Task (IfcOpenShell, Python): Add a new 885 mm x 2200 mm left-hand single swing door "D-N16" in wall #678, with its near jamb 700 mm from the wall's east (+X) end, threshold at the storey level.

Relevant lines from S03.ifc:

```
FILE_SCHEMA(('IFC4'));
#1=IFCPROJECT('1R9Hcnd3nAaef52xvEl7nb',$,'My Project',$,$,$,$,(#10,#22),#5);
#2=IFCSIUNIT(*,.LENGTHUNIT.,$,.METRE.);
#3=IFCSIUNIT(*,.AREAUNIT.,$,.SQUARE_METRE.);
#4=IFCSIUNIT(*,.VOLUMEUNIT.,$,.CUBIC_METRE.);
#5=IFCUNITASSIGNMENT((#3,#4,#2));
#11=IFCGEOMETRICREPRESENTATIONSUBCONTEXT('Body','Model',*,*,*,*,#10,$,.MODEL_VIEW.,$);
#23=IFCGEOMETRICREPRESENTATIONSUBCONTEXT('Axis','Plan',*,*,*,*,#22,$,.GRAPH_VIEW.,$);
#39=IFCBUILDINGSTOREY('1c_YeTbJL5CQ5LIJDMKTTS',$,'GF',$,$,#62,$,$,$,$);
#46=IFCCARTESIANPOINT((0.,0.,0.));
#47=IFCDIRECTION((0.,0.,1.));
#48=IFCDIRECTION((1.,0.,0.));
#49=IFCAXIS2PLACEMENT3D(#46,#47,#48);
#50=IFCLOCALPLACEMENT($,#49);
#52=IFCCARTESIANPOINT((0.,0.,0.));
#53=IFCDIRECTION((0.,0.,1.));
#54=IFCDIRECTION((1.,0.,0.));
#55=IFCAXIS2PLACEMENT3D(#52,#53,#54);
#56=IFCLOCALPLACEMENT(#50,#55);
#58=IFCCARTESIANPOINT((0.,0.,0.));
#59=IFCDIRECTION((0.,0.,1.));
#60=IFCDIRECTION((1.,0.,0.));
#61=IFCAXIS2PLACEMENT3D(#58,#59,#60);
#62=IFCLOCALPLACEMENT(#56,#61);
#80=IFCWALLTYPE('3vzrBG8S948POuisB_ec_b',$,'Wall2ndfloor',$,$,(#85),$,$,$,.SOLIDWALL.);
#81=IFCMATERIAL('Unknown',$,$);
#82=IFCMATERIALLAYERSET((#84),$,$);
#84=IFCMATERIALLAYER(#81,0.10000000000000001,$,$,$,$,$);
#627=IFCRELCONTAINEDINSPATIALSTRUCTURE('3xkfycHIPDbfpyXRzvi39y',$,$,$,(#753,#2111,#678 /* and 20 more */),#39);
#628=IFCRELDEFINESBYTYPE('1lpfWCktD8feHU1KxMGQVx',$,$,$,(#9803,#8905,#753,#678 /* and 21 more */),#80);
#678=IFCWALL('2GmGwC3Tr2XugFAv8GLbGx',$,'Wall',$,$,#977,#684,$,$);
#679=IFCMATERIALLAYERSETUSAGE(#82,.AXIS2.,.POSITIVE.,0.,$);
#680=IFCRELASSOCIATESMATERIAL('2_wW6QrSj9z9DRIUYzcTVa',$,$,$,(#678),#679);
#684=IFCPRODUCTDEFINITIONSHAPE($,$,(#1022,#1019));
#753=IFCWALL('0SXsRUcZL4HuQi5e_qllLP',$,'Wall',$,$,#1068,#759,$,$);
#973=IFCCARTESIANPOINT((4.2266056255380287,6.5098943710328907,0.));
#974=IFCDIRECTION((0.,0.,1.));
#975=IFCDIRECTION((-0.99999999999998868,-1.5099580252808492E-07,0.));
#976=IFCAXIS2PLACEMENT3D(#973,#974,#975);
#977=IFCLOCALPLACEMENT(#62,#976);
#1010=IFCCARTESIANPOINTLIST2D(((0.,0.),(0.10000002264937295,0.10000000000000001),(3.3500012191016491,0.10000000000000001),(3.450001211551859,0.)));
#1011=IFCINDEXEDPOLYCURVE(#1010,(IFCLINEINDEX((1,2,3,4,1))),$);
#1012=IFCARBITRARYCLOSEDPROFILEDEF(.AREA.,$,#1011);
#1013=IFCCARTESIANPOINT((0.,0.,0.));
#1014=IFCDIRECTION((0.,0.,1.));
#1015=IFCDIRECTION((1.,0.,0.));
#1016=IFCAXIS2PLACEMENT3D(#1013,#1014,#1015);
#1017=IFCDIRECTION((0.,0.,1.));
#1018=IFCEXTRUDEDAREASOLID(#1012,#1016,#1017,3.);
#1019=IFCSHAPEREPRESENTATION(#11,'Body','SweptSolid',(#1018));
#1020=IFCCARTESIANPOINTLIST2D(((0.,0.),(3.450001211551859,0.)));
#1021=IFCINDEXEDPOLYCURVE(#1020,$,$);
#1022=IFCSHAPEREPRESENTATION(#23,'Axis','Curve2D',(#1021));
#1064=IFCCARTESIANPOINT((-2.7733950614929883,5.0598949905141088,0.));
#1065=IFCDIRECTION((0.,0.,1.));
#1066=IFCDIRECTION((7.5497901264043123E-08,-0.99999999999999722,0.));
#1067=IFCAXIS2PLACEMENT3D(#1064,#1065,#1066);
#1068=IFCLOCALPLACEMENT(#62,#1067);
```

```python
import numpy as np
import ifcopenshell
import ifcopenshell.api.feature
import ifcopenshell.api.geometry
import ifcopenshell.api.root
import ifcopenshell.api.spatial
import ifcopenshell.geom
import ifcopenshell.util.element
import ifcopenshell.util.placement
import ifcopenshell.util.representation
import ifcopenshell.util.shape
import ifcopenshell.util.unit

model = ifcopenshell.open("S03.ifc")
unit_scale = ifcopenshell.util.unit.calculate_unit_scale(model)
settings = ifcopenshell.geom.settings()


def volume(element):
    """Net volume in cubic metres, openings subtracted."""
    shape = ifcopenshell.geom.create_shape(settings, element)
    return ifcopenshell.util.shape.get_volume(shape.geometry)


wall = model.by_guid("2GmGwC3Tr2XugFAv8GLbGx")
storey = ifcopenshell.util.element.get_container(wall, ifc_class="IfcBuildingStorey")
context = ifcopenshell.util.representation.get_context(model, "Model", "Body", "MODEL_VIEW")
before = volume(wall)

width, height, from_end, sill = 0.885, 2.2, 0.7, 0.0  # metres

# The wall runs along its own X axis, and the end named is its -X end.
wall_shape = ifcopenshell.geom.create_shape(settings, wall)
x, y, z = ifcopenshell.util.shape.get_vertices(wall_shape.geometry).T
start = x.min() + from_end
face, thickness = float(y.min()), float(y.max() - y.min())
wall_matrix = ifcopenshell.util.placement.get_local_placement(wall.ObjectPlacement)
level = ifcopenshell.util.placement.get_local_placement(storey.ObjectPlacement)[2, 3]


def in_wall(x, y):
    """Placement at x, y metres in the wall's axes, at sill height."""
    matrix = wall_matrix.copy()
    matrix[:, 3] = wall_matrix @ np.array([x / unit_scale, y / unit_scale, 0.0, 1.0])
    matrix[2, 3] = level + sill / unit_scale
    return matrix


# Opening: a box that overshoots both wall faces by 50 mm.
opening = ifcopenshell.api.root.create_entity(model, ifc_class="IfcOpeningElement", predefined_type="OPENING")
box = ifcopenshell.api.geometry.add_wall_representation(
    model, context=context, length=width, height=height, thickness=thickness + 0.1
)
ifcopenshell.api.geometry.assign_representation(model, product=opening, representation=box)
ifcopenshell.api.geometry.edit_object_placement(model, product=opening, matrix=in_wall(start, face - 0.05), is_si=False)
ifcopenshell.api.feature.add_feature(model, feature=opening, element=wall)

door = ifcopenshell.api.root.create_entity(model, ifc_class="IfcDoor", name="D-N16", predefined_type="DOOR")
door.OverallWidth, door.OverallHeight = width / unit_scale, height / unit_scale
door.OperationType = "SINGLE_SWING_LEFT"
body = ifcopenshell.api.geometry.add_door_representation(
    model,
    context=context,
    overall_width=door.OverallWidth,
    overall_height=door.OverallHeight,
    operation_type="SINGLE_SWING_LEFT",
    lining_properties={"LiningDepth": thickness / unit_scale, "ThresholdDepth": thickness / unit_scale},
)
ifcopenshell.api.geometry.assign_representation(model, product=door, representation=body)
ifcopenshell.api.spatial.assign_container(model, products=[door], relating_structure=storey)
ifcopenshell.api.feature.add_filling(model, opening=opening, element=door)

# The lining spans the wall, so the door starts at the wall face.
ifcopenshell.api.geometry.edit_object_placement(model, product=door, matrix=in_wall(start, face), is_si=False)

after = volume(wall)

print(f"wall volume {before:.3f} -> {after:.3f} m3")

model.write("S03_edited.ifc")
```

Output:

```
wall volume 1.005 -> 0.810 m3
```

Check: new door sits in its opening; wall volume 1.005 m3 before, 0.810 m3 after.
